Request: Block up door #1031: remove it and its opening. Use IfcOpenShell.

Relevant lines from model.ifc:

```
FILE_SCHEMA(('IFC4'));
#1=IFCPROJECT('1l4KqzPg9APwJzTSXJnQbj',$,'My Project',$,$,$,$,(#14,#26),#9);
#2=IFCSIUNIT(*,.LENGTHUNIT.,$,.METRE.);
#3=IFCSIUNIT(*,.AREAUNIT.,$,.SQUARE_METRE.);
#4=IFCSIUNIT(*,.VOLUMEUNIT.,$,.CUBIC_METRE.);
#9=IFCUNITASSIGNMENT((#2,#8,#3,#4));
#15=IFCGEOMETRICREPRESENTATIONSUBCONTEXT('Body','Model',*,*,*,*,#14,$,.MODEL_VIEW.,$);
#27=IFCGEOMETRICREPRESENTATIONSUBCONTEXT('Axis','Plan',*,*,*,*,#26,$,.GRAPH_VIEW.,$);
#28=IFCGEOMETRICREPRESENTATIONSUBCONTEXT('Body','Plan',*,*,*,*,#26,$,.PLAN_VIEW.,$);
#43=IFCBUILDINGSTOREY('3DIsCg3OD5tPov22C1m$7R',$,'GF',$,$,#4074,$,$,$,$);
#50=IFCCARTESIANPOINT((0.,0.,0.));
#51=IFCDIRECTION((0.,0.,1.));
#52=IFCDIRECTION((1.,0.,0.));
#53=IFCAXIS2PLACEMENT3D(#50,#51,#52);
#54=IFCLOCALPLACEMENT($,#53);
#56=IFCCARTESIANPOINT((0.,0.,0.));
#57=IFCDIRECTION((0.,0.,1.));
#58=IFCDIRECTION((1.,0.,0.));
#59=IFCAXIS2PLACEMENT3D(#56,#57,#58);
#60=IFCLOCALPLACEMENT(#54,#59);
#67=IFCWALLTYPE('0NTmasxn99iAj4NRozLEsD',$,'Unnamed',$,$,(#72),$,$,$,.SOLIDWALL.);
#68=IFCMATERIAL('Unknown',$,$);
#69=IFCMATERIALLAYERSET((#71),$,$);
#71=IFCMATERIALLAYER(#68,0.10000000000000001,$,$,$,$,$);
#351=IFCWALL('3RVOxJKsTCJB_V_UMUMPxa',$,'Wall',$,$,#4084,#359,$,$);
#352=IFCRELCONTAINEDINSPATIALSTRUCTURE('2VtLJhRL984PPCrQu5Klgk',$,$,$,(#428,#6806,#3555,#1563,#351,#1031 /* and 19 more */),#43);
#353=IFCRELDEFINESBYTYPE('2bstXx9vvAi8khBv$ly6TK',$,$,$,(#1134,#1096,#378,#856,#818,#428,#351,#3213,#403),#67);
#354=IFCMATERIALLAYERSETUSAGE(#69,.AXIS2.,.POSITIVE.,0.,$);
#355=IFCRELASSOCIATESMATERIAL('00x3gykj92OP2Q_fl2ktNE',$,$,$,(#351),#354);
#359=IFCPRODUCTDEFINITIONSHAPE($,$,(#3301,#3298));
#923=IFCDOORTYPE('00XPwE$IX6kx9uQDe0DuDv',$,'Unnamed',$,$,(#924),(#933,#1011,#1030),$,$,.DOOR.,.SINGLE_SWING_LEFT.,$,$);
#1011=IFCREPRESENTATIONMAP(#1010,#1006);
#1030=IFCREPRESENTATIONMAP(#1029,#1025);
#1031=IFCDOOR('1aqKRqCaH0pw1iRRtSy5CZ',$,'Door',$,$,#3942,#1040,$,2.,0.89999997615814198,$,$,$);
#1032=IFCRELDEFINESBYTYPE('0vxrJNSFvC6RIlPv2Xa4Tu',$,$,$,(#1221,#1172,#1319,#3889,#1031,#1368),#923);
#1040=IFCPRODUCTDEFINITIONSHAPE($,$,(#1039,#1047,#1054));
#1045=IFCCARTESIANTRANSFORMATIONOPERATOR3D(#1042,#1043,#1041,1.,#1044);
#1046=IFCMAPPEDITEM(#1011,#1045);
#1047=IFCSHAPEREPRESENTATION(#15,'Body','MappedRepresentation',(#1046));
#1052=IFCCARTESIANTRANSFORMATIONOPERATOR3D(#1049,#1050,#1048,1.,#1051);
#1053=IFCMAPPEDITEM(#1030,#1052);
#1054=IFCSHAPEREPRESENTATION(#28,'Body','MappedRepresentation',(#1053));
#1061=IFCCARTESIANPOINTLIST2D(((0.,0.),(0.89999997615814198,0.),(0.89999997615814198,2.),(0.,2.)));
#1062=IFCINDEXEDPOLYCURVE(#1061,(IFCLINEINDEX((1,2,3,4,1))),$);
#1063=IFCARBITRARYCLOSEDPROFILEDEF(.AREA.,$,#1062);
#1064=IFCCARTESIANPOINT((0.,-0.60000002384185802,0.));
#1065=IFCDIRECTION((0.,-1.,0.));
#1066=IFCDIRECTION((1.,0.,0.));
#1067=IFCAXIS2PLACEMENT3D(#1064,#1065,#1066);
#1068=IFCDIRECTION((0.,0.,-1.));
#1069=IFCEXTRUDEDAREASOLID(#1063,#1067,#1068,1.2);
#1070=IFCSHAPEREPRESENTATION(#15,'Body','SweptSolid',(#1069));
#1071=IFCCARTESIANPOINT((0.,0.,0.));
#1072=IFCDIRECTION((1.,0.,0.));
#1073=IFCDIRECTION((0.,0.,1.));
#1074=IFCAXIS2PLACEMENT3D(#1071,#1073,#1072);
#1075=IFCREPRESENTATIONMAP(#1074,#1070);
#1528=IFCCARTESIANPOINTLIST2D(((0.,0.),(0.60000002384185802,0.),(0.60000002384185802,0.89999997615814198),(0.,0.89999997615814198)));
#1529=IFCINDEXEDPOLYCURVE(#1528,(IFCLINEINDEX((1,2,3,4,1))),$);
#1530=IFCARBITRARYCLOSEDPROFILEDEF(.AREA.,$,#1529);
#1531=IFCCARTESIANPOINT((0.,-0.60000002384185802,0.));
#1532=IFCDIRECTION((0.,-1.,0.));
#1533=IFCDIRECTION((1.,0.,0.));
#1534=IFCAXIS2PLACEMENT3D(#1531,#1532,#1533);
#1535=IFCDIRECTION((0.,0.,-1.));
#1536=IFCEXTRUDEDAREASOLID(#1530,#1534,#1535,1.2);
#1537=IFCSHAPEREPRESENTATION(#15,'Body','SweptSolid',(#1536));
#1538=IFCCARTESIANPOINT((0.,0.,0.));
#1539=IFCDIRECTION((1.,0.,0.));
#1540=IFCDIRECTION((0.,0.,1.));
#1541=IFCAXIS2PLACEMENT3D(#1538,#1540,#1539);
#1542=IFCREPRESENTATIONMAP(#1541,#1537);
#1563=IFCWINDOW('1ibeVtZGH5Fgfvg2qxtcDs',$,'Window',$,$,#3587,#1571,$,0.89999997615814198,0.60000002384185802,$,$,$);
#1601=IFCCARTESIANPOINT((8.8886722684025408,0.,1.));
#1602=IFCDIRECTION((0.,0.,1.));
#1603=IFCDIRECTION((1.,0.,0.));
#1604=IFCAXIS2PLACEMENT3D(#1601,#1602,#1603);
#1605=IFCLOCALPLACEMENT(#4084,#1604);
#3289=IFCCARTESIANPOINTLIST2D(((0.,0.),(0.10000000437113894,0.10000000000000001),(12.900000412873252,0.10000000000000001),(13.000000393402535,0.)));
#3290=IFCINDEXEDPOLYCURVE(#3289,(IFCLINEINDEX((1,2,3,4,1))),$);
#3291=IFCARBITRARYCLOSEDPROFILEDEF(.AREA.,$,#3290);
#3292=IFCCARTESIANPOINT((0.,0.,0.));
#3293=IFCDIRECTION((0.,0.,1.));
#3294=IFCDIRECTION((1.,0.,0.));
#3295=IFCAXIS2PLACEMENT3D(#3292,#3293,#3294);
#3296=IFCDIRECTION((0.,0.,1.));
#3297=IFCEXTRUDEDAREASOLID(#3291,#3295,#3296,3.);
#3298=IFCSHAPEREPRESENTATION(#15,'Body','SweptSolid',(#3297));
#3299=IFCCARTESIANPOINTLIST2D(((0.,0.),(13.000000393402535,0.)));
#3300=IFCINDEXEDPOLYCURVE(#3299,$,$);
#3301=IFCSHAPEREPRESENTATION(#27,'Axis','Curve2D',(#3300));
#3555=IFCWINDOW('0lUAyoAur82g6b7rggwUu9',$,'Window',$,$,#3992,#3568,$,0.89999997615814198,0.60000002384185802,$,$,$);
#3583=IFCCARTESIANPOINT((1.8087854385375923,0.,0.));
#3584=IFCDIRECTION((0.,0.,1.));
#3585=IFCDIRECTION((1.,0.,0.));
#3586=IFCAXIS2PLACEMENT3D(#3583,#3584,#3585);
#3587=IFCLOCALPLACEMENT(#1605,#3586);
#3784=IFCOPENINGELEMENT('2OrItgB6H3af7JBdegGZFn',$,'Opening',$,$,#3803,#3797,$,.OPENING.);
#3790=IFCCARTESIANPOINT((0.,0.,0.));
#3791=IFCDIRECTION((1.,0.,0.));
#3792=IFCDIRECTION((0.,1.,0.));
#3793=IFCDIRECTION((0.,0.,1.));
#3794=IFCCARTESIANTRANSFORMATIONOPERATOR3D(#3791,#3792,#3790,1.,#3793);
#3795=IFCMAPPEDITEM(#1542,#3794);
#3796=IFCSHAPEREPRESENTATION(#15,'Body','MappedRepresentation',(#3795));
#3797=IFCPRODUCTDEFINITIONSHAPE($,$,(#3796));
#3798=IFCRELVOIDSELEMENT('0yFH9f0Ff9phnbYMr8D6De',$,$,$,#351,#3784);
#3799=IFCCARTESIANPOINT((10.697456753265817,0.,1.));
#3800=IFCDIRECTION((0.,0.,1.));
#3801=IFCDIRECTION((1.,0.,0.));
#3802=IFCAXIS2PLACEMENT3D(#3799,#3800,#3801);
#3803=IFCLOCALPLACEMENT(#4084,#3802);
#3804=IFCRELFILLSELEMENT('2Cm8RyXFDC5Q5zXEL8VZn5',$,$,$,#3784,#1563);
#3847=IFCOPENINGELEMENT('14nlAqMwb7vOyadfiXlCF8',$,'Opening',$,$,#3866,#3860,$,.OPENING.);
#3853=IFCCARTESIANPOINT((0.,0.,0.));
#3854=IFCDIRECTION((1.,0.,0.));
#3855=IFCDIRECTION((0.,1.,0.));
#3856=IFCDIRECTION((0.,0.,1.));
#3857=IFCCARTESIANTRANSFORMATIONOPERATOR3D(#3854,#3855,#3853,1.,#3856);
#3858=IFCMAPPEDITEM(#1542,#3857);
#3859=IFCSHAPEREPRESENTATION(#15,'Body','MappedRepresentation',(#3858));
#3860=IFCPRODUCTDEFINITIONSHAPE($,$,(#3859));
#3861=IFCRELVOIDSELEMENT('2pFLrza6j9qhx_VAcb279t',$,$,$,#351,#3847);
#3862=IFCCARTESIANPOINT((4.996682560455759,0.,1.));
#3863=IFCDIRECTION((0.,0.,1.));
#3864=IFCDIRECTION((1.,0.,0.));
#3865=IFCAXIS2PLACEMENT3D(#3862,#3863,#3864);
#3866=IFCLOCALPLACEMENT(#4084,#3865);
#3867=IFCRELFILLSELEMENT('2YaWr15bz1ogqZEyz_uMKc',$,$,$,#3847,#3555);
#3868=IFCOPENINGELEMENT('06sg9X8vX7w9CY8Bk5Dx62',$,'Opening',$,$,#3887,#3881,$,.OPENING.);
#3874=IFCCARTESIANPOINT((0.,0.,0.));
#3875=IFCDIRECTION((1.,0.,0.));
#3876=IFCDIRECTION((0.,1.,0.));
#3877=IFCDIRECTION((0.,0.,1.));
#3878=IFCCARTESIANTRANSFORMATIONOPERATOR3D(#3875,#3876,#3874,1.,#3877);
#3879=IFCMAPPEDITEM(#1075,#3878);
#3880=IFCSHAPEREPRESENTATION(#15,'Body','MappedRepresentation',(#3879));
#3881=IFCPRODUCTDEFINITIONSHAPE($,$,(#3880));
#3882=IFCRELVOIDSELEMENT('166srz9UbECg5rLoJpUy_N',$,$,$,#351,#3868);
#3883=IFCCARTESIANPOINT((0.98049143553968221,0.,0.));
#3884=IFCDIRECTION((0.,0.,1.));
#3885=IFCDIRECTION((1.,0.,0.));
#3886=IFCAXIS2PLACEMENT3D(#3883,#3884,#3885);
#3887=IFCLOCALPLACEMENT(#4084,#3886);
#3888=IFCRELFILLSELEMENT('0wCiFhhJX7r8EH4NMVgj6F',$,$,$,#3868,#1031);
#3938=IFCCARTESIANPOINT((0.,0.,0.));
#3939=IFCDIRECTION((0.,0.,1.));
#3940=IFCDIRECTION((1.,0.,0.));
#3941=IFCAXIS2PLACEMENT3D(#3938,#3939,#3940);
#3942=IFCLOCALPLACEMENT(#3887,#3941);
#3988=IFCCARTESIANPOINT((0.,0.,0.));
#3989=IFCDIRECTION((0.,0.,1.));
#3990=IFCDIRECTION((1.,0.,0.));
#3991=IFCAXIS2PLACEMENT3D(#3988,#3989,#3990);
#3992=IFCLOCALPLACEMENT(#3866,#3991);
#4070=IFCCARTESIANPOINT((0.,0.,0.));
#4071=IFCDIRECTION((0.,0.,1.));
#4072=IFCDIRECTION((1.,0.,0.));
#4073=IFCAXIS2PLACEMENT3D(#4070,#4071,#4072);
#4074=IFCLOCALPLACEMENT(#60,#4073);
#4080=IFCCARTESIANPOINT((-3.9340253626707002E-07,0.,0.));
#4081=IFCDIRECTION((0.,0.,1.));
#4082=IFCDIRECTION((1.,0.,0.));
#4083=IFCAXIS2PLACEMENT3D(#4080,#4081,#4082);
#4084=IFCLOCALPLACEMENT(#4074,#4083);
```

```python
import ifcopenshell
import ifcopenshell.api.feature
import ifcopenshell.api.root
import ifcopenshell.geom
import ifcopenshell.util.shape

model = ifcopenshell.open("model.ifc")
settings = ifcopenshell.geom.settings()


def volume(element):
    """Net volume in cubic metres, openings subtracted."""
    shape = ifcopenshell.geom.create_shape(settings, element)
    return ifcopenshell.util.shape.get_volume(shape.geometry)


door = model.by_guid("1aqKRqCaH0pw1iRRtSy5CZ")
opening = door.FillsVoids[0].RelatingOpeningElement
wall = opening.VoidsElements[0].RelatingBuildingElement
before = volume(wall)

ifcopenshell.api.root.remove_product(model, product=door)
ifcopenshell.api.feature.remove_feature(model, feature=opening)

after = volume(wall)

print(f"wall volume {before:.3f} -> {after:.3f} m3")

model.write("model_v2.ifc")
```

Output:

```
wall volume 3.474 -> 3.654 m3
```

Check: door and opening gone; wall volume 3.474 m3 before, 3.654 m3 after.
